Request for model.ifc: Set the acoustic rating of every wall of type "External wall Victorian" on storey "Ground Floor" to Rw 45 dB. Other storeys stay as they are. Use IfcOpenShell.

First a look at what the model holds.

```python
import ifcopenshell
import ifcopenshell.util.element

model = ifcopenshell.open("model.ifc")
print(model.schema)
storey = next(s for s in model.by_type("IfcBuildingStorey") if s.Name == "Ground Floor")
walls = [e for e in ifcopenshell.util.element.get_decomposition(storey) if e.is_a("IfcWall")]
seen = {}
for e in walls:
    element_type = ifcopenshell.util.element.get_type(e)
    key = (element_type.Name if element_type != e and element_type else None, ifcopenshell.util.element.get_pset(e, "Pset_WallCommon", "AcousticRating"))
    seen[key] = seen.get(key, 0) + 1
for (name, value), count in sorted(seen.items(), key=str):
    print(count, "x", name, "|", value)
```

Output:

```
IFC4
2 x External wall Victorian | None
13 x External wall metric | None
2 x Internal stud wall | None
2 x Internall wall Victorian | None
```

```python
import ifcopenshell
import ifcopenshell.api.pset
import ifcopenshell.util.element

model = ifcopenshell.open("model.ifc")

storey = next(s for s in model.by_type("IfcBuildingStorey") if s.Name == "Ground Floor")
walls = [e for e in ifcopenshell.util.element.get_decomposition(storey) if e.is_a("IfcWall")]

count = 0
for e in walls:
    element_type = ifcopenshell.util.element.get_type(e)
    if element_type in (None, e) or element_type.Name != "External wall Victorian":
        continue
    # add_pset returns the element's existing set when there is one.
    pset = ifcopenshell.api.pset.add_pset(model, product=e, name="Pset_WallCommon")
    ifcopenshell.api.pset.edit_pset(model, pset=pset, properties={"AcousticRating": "Rw 45 dB"})
    count += 1

print(count, "walls updated")

model.write("model-out.ifc")
```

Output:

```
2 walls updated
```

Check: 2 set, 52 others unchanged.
